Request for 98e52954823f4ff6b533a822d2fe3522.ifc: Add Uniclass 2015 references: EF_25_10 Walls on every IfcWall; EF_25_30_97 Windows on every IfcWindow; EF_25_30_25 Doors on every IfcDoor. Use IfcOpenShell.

First a look at what the model holds.

```python
import ifcopenshell

model = ifcopenshell.open("98e52954823f4ff6b533a822d2fe3522.ifc")
print(model.schema)
print("classifications:", [c.Name for c in model.by_type("IfcClassification")])
for ifc_class in ("IfcDoor", "IfcRoof", "IfcStair", "IfcWall", "IfcWindow"):
    print(ifc_class, len(model.by_type(ifc_class)))
```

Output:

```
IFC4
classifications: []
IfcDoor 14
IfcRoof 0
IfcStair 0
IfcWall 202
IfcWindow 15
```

```python
import ifcopenshell
import ifcopenshell.api.classification

model = ifcopenshell.open("98e52954823f4ff6b533a822d2fe3522.ifc")

system = ifcopenshell.api.classification.add_classification(model, classification="Uniclass 2015")

codes = {
    "IfcWall": ("EF_25_10", "Walls"),
    "IfcWindow": ("EF_25_30_97", "Windows"),
    "IfcDoor": ("EF_25_30_25", "Doors"),
}
for ifc_class, (code, name) in codes.items():
    products = model.by_type(ifc_class)
    ifcopenshell.api.classification.add_reference(
        model, products=products, classification=system, identification=code, name=name
    )
    print(code, len(products))

model.write("98e52954823f4ff6b533a822d2fe3522_v2.ifc")
```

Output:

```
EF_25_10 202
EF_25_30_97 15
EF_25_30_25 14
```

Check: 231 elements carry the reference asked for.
